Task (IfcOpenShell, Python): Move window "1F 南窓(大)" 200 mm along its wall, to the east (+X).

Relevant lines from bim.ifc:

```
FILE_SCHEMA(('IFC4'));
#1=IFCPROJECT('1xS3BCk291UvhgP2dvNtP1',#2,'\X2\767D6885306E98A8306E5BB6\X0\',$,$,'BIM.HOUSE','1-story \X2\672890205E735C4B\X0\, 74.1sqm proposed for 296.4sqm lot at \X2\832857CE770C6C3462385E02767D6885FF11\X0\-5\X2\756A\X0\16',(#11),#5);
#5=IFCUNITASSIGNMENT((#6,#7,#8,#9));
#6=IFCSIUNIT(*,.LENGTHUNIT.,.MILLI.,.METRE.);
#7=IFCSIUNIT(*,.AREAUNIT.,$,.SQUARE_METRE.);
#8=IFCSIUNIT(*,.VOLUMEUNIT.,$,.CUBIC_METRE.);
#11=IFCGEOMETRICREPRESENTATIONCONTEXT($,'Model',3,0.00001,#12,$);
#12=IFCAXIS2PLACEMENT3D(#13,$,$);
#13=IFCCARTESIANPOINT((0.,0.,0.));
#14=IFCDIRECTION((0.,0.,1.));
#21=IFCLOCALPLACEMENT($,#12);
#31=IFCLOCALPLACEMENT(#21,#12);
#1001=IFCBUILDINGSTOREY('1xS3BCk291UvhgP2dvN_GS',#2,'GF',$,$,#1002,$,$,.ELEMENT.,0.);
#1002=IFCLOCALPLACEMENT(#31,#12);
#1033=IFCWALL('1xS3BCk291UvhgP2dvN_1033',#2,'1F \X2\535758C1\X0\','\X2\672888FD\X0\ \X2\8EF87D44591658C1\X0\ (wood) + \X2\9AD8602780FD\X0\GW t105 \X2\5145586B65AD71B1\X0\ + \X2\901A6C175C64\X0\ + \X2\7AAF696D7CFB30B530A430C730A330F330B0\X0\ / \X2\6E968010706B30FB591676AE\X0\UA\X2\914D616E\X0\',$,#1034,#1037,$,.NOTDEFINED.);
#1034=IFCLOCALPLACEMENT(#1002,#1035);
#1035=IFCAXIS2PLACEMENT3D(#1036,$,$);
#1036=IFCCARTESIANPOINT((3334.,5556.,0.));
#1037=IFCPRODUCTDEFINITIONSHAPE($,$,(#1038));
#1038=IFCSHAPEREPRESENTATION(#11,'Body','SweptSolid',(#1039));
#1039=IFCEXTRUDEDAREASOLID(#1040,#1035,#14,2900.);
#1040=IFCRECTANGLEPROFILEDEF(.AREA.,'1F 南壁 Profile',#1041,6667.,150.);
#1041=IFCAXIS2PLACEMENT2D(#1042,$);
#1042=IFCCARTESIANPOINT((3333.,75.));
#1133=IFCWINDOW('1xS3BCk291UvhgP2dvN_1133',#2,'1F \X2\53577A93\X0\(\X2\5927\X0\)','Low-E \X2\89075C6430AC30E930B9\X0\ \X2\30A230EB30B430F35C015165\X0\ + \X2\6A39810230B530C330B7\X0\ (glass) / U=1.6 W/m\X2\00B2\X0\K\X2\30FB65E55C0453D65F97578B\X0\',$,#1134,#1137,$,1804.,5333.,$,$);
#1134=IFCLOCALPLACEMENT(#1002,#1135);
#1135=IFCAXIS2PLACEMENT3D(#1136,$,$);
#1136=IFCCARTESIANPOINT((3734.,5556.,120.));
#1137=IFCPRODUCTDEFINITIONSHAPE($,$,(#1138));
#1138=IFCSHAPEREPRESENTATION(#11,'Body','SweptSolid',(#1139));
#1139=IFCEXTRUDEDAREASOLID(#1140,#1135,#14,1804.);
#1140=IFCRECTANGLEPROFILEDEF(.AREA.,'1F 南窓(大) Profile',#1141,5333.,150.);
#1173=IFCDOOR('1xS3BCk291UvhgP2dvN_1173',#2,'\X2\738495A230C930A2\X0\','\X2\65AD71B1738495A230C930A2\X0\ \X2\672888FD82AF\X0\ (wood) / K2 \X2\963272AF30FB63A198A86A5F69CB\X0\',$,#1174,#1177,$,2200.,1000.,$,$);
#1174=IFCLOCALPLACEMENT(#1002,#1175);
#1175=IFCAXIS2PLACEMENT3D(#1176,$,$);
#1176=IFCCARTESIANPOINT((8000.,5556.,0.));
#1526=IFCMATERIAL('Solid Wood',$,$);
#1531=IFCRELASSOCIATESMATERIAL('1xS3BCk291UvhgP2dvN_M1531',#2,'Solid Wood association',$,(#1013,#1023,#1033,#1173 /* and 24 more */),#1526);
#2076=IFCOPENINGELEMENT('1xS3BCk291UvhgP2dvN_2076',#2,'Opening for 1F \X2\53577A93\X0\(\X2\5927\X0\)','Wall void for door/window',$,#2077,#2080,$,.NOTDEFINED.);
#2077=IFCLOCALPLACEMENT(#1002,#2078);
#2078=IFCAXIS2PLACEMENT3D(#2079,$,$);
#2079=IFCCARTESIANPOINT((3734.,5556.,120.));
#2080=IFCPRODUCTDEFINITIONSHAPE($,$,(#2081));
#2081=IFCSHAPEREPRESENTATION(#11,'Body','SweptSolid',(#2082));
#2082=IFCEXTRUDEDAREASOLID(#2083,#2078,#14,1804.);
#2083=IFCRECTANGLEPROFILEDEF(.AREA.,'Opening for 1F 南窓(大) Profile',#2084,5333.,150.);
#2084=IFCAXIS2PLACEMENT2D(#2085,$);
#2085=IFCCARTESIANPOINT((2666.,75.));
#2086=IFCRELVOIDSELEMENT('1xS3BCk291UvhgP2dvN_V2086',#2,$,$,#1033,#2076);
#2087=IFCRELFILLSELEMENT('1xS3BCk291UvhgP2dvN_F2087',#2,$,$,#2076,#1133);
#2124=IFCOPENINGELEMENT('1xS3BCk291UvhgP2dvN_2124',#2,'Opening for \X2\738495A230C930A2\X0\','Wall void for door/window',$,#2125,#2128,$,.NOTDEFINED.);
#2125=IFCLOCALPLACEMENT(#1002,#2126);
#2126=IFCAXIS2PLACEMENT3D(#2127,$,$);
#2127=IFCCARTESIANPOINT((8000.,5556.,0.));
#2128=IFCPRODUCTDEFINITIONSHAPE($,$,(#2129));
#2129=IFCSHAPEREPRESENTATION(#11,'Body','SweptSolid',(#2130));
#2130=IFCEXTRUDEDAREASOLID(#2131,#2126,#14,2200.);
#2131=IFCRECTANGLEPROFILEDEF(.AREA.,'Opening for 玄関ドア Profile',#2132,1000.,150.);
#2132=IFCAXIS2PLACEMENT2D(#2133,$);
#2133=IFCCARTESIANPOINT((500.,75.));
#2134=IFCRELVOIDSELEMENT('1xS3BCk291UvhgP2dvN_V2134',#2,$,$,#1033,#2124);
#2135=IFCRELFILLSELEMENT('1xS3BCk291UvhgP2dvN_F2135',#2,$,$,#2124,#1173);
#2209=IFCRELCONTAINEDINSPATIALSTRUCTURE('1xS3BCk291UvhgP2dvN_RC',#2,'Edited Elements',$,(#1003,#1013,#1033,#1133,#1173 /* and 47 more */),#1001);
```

```python
import ifcopenshell
import ifcopenshell.api.geometry
import ifcopenshell.util.placement

model = ifcopenshell.open("bim.ifc")

window = model.by_guid("1xS3BCk291UvhgP2dvN_1133")
opening = window.FillsVoids[0].RelatingOpeningElement
wall = opening.VoidsElements[0].RelatingBuildingElement

wall_matrix = ifcopenshell.util.placement.get_local_placement(wall.ObjectPlacement)
shift = wall_matrix[:3, 0] * 200.0
before = ifcopenshell.util.placement.get_local_placement(window.ObjectPlacement)[:3, 3].copy()

# The window is not placed relative to its opening, so move both.
for product in (opening, window):
    matrix = ifcopenshell.util.placement.get_local_placement(product.ObjectPlacement)
    matrix[:3, 3] += shift
    ifcopenshell.api.geometry.edit_object_placement(model, product=product, matrix=matrix, is_si=False)

after = ifcopenshell.util.placement.get_local_placement(window.ObjectPlacement)[:3, 3]
print("window moved by", (after - before).round(3) + 0.0)

model.write("bim_updated.ifc")
```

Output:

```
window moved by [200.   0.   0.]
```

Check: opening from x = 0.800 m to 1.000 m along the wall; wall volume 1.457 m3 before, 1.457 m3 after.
